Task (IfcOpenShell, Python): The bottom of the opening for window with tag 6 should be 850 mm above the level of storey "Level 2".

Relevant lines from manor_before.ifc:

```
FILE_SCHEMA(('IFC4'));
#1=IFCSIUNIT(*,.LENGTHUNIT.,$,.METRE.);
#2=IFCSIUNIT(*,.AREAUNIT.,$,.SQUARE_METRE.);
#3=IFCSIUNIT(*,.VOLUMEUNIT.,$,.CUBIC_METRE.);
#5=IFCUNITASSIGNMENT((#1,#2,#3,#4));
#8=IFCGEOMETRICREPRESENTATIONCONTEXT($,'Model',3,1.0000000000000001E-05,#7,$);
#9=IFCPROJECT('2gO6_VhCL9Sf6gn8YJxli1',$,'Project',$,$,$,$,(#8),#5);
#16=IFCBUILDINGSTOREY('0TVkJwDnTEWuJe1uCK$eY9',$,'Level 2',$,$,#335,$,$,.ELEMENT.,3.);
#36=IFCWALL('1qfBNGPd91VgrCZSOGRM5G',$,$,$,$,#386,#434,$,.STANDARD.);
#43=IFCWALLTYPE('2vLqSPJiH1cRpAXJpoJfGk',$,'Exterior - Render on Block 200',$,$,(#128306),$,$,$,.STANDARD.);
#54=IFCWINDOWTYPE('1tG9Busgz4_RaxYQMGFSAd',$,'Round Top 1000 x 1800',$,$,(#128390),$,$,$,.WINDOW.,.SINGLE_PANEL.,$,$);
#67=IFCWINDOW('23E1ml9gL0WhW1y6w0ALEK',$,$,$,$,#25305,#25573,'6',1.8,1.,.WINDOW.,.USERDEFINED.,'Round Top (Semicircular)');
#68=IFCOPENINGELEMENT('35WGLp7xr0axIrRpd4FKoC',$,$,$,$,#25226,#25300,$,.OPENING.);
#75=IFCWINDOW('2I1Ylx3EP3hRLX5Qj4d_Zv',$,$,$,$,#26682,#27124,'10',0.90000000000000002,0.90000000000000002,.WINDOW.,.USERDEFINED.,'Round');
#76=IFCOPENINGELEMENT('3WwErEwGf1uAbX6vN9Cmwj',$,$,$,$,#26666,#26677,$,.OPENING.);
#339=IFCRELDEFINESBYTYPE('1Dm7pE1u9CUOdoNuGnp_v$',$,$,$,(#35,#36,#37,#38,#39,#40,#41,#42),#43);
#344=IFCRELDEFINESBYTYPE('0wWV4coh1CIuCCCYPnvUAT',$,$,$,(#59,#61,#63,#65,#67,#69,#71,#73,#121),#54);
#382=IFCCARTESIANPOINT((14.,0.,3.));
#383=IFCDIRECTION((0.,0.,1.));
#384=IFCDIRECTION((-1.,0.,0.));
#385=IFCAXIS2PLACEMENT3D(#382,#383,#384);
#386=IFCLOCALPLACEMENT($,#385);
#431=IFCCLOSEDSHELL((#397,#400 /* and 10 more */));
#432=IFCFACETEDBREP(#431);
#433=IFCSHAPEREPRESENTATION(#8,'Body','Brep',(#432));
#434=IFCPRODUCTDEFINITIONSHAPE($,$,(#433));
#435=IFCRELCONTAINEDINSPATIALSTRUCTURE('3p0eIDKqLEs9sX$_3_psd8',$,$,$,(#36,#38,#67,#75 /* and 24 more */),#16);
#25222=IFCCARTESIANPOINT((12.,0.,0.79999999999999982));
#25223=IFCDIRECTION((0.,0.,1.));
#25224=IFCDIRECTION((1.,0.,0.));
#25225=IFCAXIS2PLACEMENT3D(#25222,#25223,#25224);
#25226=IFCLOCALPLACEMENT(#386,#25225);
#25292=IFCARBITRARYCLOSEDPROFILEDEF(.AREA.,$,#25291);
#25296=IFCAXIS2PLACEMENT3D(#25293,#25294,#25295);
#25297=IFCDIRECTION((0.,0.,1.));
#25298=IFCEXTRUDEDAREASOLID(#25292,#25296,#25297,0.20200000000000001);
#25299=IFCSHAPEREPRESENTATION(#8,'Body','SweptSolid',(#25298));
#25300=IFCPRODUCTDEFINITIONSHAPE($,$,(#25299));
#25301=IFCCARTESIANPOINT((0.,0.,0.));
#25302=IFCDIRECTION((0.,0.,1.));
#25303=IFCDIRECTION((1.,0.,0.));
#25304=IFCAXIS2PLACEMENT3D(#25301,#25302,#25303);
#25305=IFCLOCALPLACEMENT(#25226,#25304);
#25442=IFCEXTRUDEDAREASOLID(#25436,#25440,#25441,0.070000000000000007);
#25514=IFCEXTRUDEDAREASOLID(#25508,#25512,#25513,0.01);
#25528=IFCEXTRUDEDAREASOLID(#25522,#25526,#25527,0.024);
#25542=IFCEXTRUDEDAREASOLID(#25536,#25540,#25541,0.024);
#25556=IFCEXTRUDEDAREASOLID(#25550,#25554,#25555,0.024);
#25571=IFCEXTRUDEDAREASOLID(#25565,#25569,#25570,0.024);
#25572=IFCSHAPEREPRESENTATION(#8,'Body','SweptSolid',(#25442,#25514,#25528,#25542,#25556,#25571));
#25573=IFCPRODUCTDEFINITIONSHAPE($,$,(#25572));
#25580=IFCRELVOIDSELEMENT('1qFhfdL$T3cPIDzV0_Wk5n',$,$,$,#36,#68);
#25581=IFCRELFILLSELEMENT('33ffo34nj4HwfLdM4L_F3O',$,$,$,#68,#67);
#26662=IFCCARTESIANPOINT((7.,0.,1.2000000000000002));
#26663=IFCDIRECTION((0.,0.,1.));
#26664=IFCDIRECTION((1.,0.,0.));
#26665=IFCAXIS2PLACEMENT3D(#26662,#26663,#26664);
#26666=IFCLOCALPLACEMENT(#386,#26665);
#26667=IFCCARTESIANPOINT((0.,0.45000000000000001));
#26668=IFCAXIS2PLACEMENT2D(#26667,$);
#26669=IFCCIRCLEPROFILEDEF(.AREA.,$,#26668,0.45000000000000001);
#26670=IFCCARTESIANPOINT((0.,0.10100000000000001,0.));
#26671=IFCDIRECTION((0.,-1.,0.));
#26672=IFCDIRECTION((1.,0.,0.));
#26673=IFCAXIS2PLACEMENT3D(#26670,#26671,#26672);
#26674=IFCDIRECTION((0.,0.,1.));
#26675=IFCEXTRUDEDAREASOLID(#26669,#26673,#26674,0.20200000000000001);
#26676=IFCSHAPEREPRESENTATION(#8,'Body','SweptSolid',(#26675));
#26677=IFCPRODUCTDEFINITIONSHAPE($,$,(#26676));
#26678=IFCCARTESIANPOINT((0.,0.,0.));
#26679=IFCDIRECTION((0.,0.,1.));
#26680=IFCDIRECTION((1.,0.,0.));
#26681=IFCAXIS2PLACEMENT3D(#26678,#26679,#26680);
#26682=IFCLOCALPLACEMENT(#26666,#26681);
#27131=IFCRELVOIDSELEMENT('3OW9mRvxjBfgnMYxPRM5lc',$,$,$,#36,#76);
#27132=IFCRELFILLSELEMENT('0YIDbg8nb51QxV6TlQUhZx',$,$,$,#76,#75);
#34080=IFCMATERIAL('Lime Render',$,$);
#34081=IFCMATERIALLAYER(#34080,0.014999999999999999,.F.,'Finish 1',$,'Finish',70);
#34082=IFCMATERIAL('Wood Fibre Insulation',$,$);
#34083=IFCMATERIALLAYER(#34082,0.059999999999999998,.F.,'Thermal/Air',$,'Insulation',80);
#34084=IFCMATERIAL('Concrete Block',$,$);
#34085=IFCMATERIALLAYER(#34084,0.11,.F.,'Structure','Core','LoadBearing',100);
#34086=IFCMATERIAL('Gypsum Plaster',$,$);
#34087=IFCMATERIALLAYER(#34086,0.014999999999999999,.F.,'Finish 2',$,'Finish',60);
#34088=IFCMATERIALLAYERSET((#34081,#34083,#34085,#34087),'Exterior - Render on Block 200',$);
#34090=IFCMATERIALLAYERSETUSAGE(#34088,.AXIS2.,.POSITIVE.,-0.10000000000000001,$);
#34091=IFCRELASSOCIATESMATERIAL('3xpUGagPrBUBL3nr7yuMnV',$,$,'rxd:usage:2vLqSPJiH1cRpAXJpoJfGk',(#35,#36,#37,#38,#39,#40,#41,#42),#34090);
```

```python
import numpy as np
import ifcopenshell
import ifcopenshell.api.geometry
import ifcopenshell.geom
import ifcopenshell.util.element
import ifcopenshell.util.placement
import ifcopenshell.util.shape
import ifcopenshell.util.unit

model = ifcopenshell.open("manor_before.ifc")
unit_scale = ifcopenshell.util.unit.calculate_unit_scale(model)

window = model.by_id(67)
opening = window.FillsVoids[0].RelatingOpeningElement
storey = ifcopenshell.util.element.get_container(window, ifc_class="IfcBuildingStorey")
level = ifcopenshell.util.placement.get_local_placement(storey.ObjectPlacement)[2, 3]

# The opening's origin need not be at the sill, so measure its lowest point.
shape = ifcopenshell.geom.create_shape(ifcopenshell.geom.settings(), opening)
bottom = ifcopenshell.util.shape.get_shape_bottom_elevation(shape, shape.geometry) / unit_scale
dz = level + 0.85 / unit_scale - bottom

shift = np.array([0.0, 0.0, dz])
# The window is placed relative to its opening, so it follows when the opening moves.
matrix = ifcopenshell.util.placement.get_local_placement(opening.ObjectPlacement)
matrix[:3, 3] += shift
ifcopenshell.api.geometry.edit_object_placement(
    model, product=opening, matrix=matrix, is_si=False, should_transform_children=True
)

print(f"moved by {dz * unit_scale:+.3f} m")

model.write("manor_before-out.ifc")
```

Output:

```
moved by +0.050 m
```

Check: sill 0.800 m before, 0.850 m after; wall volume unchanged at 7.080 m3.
